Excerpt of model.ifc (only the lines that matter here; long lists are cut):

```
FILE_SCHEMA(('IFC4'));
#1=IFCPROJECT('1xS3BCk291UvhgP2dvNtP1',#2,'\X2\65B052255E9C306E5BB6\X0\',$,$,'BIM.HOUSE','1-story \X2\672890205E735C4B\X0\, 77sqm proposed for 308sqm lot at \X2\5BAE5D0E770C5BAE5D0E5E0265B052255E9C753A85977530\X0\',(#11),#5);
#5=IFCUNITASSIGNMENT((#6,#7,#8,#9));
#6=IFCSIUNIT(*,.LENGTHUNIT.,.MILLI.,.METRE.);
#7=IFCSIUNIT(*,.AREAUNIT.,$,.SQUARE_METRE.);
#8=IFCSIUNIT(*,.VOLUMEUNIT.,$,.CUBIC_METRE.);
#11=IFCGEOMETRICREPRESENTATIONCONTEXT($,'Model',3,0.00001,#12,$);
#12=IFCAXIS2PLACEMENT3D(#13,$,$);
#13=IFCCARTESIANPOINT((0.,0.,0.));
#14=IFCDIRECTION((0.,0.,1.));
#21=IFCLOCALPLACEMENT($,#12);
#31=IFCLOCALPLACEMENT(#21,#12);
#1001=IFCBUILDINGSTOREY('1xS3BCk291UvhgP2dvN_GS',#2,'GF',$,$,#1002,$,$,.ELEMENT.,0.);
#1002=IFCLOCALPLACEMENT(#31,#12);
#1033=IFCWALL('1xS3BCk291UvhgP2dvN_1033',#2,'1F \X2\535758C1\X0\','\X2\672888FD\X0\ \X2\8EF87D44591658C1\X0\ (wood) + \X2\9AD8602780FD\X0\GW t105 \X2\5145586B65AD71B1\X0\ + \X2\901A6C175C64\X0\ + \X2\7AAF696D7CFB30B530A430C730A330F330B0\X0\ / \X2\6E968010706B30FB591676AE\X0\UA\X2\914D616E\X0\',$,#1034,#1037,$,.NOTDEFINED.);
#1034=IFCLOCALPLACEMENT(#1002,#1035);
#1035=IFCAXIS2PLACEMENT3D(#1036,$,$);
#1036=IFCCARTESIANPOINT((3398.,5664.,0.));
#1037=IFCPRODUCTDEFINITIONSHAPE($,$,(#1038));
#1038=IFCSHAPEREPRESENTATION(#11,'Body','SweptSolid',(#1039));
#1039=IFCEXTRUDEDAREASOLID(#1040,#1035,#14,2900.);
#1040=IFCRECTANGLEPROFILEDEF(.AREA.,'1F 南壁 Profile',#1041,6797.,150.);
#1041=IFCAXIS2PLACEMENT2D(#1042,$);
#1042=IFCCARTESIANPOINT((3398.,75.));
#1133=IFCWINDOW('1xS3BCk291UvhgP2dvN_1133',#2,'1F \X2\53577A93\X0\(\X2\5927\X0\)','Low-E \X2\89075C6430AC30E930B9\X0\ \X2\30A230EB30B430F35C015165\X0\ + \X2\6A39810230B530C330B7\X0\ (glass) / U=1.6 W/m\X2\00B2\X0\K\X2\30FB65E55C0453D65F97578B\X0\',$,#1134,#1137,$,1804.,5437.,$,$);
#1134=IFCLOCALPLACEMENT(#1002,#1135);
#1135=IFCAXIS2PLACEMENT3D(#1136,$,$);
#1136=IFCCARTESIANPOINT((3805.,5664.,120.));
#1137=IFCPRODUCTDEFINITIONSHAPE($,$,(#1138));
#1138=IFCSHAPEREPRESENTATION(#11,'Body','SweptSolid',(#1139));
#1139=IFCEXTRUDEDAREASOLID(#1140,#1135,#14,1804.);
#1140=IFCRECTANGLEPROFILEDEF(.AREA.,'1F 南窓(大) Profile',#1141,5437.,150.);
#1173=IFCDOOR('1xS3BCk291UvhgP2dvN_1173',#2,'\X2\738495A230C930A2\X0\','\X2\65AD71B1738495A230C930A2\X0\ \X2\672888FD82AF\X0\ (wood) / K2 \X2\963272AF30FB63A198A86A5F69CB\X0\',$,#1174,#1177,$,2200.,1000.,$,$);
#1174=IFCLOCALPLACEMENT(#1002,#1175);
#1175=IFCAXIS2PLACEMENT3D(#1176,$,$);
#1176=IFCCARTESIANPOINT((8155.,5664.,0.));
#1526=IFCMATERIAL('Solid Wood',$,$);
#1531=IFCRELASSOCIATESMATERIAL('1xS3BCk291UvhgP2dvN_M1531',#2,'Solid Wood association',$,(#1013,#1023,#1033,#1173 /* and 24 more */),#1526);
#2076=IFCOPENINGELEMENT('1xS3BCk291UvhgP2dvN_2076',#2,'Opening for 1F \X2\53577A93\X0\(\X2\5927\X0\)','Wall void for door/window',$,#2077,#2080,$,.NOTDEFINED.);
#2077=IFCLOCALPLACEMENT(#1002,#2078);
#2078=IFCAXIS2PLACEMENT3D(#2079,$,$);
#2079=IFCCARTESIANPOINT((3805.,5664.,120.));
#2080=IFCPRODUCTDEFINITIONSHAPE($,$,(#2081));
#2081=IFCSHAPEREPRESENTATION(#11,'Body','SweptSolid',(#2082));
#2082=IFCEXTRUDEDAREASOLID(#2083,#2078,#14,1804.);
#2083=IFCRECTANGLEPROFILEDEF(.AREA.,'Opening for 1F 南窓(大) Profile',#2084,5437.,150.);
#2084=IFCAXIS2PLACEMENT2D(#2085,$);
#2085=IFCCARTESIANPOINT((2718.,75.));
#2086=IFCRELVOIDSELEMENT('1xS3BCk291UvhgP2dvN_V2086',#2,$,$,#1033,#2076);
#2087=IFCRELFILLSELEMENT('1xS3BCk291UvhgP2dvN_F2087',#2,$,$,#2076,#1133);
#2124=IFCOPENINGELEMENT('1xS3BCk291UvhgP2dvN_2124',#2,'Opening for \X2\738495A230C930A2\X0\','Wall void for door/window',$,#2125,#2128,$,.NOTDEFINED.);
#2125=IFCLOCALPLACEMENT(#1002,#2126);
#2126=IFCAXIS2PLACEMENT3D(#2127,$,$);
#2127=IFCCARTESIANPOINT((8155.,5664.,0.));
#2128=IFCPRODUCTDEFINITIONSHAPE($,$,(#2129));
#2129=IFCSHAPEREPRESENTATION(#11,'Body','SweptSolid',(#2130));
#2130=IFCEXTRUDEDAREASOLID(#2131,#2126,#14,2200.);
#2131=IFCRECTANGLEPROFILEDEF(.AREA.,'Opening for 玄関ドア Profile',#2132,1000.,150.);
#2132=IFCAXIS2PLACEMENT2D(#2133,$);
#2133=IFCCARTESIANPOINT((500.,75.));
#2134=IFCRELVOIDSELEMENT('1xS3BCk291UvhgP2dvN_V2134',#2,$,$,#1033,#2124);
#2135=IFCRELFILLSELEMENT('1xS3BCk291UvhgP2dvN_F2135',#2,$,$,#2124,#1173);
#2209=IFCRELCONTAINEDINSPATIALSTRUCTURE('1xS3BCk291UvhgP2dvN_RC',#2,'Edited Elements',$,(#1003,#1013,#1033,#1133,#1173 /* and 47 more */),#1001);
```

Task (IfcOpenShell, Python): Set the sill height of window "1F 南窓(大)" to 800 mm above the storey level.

```python
import numpy as np
import ifcopenshell
import ifcopenshell.api.geometry
import ifcopenshell.geom
import ifcopenshell.util.element
import ifcopenshell.util.placement
import ifcopenshell.util.shape
import ifcopenshell.util.unit

model = ifcopenshell.open("model.ifc")
unit_scale = ifcopenshell.util.unit.calculate_unit_scale(model)

window = model.by_id(1133)
opening = window.FillsVoids[0].RelatingOpeningElement
storey = ifcopenshell.util.element.get_container(window, ifc_class="IfcBuildingStorey")
level = ifcopenshell.util.placement.get_local_placement(storey.ObjectPlacement)[2, 3]

# The opening's origin need not be at the sill, so measure its lowest point.
shape = ifcopenshell.geom.create_shape(ifcopenshell.geom.settings(), opening)
bottom = ifcopenshell.util.shape.get_shape_bottom_elevation(shape, shape.geometry) / unit_scale
dz = level + 800.0 - bottom

shift = np.array([0.0, 0.0, dz])
# The window is not placed relative to its opening, so move both.
for product in (opening, window):
    matrix = ifcopenshell.util.placement.get_local_placement(product.ObjectPlacement)
    matrix[:3, 3] += shift
    ifcopenshell.api.geometry.edit_object_placement(model, product=product, matrix=matrix, is_si=False)

print(f"moved by {dz * unit_scale:+.3f} m")

model.write("model_updated.ifc")
```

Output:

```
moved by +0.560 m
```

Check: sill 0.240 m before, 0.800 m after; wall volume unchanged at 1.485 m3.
